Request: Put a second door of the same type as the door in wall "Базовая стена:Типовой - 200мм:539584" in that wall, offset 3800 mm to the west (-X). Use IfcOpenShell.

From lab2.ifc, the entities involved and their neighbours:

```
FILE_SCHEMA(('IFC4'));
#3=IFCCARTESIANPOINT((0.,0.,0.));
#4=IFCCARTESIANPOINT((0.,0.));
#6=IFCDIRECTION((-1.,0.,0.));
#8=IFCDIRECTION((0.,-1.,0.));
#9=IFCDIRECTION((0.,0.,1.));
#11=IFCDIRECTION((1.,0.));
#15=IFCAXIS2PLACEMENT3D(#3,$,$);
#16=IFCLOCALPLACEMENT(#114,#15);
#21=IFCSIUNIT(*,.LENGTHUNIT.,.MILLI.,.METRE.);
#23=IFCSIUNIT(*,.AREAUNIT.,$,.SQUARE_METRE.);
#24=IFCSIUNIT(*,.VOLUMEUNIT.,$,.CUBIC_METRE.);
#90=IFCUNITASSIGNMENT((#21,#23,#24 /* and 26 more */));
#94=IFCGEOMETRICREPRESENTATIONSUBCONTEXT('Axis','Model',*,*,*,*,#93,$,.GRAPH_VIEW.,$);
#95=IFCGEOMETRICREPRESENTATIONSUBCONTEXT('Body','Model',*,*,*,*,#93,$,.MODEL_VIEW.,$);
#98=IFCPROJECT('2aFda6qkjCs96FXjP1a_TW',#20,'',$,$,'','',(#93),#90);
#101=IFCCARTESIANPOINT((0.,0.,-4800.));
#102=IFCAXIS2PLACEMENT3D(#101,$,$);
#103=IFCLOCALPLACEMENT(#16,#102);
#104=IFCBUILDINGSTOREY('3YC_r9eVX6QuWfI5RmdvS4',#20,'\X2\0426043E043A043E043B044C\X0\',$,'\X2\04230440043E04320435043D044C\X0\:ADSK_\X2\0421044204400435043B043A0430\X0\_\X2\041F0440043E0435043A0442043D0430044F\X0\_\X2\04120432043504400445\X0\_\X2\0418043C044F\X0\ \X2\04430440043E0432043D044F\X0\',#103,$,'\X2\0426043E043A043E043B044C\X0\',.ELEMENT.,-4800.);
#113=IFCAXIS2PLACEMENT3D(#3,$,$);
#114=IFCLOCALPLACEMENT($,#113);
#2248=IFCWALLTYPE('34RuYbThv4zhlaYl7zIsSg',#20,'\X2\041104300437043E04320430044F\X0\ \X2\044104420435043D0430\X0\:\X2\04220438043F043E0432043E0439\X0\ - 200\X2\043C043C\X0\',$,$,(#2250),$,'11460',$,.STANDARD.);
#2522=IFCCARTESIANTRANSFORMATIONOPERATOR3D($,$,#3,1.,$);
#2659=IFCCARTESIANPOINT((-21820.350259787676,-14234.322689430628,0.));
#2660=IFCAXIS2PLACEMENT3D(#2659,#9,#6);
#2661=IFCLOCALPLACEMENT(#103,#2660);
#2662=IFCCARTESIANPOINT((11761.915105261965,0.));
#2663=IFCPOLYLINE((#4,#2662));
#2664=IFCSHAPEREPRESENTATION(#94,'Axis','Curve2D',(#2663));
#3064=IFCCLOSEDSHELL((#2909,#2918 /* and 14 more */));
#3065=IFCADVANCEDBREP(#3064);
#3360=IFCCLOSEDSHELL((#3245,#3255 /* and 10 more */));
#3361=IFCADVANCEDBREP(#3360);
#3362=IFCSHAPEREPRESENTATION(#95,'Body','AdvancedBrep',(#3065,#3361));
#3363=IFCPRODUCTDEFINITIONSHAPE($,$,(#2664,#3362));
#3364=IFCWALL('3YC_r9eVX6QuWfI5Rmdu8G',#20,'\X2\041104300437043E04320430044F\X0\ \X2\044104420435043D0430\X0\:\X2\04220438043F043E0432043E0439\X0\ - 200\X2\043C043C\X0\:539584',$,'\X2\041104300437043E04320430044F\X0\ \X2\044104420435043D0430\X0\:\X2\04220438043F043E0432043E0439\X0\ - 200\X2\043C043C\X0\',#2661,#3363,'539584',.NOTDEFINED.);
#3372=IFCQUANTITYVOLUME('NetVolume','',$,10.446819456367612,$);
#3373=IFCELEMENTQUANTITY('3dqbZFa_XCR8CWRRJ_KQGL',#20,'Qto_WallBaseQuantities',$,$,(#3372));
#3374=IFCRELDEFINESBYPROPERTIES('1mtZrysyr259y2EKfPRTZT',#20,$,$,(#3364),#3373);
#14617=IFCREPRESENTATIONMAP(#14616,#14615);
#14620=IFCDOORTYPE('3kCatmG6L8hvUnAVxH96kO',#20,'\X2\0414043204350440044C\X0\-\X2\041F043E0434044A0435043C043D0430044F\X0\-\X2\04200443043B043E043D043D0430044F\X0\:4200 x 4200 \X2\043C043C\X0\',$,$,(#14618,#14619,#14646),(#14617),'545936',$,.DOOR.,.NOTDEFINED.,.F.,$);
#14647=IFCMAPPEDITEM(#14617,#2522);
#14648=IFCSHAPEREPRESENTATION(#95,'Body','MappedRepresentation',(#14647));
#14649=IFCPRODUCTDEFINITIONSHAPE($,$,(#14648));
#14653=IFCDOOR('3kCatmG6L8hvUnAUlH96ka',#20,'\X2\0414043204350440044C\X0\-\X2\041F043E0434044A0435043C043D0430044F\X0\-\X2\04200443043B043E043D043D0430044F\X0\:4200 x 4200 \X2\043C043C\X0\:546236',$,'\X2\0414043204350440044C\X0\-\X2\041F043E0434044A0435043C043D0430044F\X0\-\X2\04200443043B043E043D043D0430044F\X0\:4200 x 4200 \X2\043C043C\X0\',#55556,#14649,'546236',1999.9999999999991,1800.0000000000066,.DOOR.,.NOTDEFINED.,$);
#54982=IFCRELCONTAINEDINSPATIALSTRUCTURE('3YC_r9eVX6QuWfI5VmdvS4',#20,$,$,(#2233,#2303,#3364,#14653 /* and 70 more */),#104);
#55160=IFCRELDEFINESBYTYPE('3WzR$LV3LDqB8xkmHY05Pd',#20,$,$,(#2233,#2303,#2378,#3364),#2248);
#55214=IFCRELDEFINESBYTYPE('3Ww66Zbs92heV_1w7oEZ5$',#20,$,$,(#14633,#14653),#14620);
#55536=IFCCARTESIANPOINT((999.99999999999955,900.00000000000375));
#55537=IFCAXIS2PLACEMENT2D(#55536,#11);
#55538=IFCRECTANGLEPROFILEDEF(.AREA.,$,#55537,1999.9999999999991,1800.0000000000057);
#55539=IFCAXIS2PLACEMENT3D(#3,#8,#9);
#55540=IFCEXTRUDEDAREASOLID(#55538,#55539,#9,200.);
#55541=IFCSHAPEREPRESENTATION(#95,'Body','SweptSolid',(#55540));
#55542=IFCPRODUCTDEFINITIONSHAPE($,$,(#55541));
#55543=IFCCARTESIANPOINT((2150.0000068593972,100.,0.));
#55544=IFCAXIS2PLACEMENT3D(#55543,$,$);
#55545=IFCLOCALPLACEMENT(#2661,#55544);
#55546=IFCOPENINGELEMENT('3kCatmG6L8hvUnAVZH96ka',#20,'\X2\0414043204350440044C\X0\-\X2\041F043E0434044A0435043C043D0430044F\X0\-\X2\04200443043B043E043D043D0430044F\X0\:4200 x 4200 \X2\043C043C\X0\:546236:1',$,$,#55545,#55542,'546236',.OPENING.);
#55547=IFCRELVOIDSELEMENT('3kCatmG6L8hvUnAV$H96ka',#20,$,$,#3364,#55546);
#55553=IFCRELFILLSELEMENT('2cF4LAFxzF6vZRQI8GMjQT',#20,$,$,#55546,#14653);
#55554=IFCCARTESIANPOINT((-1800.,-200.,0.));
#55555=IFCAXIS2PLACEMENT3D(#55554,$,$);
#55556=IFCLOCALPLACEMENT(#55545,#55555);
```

```python
import ifcopenshell
import ifcopenshell.api.feature
import ifcopenshell.api.geometry
import ifcopenshell.api.pset
import ifcopenshell.api.root
import ifcopenshell.geom
import ifcopenshell.util.element
import ifcopenshell.util.placement
import ifcopenshell.util.shape
import ifcopenshell.util.unit

model = ifcopenshell.open("lab2.ifc")
unit_scale = ifcopenshell.util.unit.calculate_unit_scale(model)
volume_scale = ifcopenshell.util.unit.calculate_unit_scale(model, "VOLUMEUNIT")
settings = ifcopenshell.geom.settings()


def volume(element):
    """Net volume in cubic metres, openings subtracted."""
    shape = ifcopenshell.geom.create_shape(settings, element)
    return ifcopenshell.util.shape.get_volume(shape.geometry)


def reuse_history(source, copy):
    """copy_class also copies each property set's owner history, people and application; keep the originals."""
    for rel in copy.IsDefinedBy:
        if rel.is_a("IfcRelDefinesByProperties") and (history := rel.RelatingPropertyDefinition.OwnerHistory):
            rel.RelatingPropertyDefinition.OwnerHistory = source.OwnerHistory
            ifcopenshell.util.element.remove_deep2(model, history)


door = model.by_guid("3kCatmG6L8hvUnAUlH96ka")
opening = door.FillsVoids[0].RelatingOpeningElement
wall = opening.VoidsElements[0].RelatingBuildingElement
before = volume(wall)
shift = ifcopenshell.util.placement.get_local_placement(wall.ObjectPlacement)[:3, 0] * 3.8 / unit_scale

# copy_class copies the void relationship, type, container and properties, but no geometry.
new_opening = ifcopenshell.api.root.copy_class(model, product=opening)
new_opening.Representation = ifcopenshell.util.element.copy_deep(
    model, opening.Representation, exclude=["IfcGeometricRepresentationContext", "IfcRepresentationMap"]
)
new_opening.Name = "Дверь-Подъемная-Рулонная:4200 x 4200 мм"
new_opening.Tag = None
reuse_history(opening, new_opening)
new_door = ifcopenshell.api.root.copy_class(model, product=door)
new_door.Representation = ifcopenshell.util.element.copy_deep(
    model, door.Representation, exclude=["IfcGeometricRepresentationContext", "IfcRepresentationMap"]
)
new_door.Name = "Дверь-Подъемная-Рулонная:4200 x 4200 мм"
new_door.Tag = None
reuse_history(door, new_door)
ifcopenshell.api.feature.add_filling(model, opening=new_opening, element=new_door)

for old, new in ((opening, new_opening), (door, new_door)):
    matrix = ifcopenshell.util.placement.get_local_placement(old.ObjectPlacement)
    matrix[:3, 3] += shift
    ifcopenshell.api.geometry.edit_object_placement(model, product=new, matrix=matrix, is_si=False)

after = volume(wall)

# Update the wall's stored quantities.
qto = model.by_id(ifcopenshell.util.element.get_pset(wall, "Qto_WallBaseQuantities", should_inherit=False)["id"])
ifcopenshell.api.pset.edit_qto(model, qto=qto, properties={"NetVolume": after / volume_scale})

print(f"wall volume {before:.3f} -> {after:.3f} m3")

model.write("lab2_rev.ifc")
```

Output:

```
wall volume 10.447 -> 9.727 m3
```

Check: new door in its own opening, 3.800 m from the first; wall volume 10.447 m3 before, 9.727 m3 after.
